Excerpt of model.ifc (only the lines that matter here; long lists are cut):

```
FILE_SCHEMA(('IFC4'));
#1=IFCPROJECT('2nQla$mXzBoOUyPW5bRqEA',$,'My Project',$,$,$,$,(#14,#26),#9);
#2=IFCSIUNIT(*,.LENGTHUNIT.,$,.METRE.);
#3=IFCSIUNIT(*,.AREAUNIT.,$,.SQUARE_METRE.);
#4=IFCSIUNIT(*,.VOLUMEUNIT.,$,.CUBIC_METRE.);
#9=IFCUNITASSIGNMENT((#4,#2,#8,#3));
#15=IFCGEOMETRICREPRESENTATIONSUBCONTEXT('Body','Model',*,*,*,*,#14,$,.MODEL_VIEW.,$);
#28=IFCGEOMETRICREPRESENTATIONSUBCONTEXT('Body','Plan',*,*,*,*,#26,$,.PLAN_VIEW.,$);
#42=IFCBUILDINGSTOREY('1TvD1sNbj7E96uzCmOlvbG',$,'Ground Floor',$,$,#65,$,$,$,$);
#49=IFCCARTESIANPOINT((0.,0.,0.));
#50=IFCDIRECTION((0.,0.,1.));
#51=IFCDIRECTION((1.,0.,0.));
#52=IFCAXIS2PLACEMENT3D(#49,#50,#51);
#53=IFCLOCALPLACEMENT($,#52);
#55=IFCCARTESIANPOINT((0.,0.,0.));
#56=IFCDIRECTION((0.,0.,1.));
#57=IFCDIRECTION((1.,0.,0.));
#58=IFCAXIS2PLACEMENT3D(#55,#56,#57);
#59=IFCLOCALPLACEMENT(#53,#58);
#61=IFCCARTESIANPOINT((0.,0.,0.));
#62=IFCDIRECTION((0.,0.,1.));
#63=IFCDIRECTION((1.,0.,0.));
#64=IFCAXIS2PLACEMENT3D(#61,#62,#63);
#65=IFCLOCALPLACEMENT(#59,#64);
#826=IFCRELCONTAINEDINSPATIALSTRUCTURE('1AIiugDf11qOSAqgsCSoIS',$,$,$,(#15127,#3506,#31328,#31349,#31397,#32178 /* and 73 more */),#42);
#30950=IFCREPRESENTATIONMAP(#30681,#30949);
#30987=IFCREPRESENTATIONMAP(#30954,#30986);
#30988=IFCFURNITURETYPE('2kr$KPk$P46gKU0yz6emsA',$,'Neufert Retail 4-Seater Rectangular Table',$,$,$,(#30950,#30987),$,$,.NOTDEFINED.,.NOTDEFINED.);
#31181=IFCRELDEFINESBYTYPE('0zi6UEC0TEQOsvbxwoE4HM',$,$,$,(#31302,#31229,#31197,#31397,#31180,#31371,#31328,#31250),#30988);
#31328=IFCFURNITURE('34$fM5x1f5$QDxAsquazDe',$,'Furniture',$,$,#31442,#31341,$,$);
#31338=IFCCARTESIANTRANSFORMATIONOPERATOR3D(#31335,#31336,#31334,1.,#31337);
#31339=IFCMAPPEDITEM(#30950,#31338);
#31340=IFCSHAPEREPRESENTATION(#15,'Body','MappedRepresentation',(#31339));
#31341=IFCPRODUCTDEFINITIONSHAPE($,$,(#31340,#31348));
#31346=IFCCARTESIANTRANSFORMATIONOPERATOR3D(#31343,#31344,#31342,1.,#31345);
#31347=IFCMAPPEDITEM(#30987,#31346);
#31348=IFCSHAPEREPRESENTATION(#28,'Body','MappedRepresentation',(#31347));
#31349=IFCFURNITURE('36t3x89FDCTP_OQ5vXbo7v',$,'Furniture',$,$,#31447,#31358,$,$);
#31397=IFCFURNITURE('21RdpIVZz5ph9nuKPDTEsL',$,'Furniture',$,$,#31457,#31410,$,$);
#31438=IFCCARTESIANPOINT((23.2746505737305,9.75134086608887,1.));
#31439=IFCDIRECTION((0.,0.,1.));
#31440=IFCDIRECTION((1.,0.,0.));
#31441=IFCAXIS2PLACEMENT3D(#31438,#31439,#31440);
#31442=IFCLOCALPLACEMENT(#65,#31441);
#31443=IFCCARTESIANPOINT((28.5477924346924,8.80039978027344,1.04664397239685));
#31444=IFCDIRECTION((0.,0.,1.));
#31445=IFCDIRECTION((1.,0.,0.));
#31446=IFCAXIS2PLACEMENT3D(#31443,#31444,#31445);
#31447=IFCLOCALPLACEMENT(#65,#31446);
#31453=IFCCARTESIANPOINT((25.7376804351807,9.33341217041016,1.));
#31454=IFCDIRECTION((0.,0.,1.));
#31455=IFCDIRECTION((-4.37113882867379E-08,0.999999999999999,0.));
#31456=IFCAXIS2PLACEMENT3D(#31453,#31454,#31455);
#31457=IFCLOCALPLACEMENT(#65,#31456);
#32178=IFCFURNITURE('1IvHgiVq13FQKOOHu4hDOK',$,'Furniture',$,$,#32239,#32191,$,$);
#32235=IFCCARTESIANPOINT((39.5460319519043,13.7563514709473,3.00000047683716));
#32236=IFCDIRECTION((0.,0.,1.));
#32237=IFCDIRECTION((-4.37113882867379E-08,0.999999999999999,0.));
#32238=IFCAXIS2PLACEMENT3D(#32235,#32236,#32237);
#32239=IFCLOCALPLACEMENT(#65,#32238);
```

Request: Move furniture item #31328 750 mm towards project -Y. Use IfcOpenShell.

```python
import ifcopenshell
import ifcopenshell.api.geometry
import ifcopenshell.util.placement
import ifcopenshell.util.unit

model = ifcopenshell.open("model.ifc")
unit_scale = ifcopenshell.util.unit.calculate_unit_scale(model)

item = model.by_guid("34$fM5x1f5$QDxAsquazDe")
matrix = ifcopenshell.util.placement.get_local_placement(item.ObjectPlacement)
matrix[1, 3] -= 0.75 / unit_scale
ifcopenshell.api.geometry.edit_object_placement(model, product=item, matrix=matrix, is_si=False)

print(ifcopenshell.util.placement.get_local_placement(item.ObjectPlacement).round(3) + 0.0)

model.write("model_v2.ifc")
```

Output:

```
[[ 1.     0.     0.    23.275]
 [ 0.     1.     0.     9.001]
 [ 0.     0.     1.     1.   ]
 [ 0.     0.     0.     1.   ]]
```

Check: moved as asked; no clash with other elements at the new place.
